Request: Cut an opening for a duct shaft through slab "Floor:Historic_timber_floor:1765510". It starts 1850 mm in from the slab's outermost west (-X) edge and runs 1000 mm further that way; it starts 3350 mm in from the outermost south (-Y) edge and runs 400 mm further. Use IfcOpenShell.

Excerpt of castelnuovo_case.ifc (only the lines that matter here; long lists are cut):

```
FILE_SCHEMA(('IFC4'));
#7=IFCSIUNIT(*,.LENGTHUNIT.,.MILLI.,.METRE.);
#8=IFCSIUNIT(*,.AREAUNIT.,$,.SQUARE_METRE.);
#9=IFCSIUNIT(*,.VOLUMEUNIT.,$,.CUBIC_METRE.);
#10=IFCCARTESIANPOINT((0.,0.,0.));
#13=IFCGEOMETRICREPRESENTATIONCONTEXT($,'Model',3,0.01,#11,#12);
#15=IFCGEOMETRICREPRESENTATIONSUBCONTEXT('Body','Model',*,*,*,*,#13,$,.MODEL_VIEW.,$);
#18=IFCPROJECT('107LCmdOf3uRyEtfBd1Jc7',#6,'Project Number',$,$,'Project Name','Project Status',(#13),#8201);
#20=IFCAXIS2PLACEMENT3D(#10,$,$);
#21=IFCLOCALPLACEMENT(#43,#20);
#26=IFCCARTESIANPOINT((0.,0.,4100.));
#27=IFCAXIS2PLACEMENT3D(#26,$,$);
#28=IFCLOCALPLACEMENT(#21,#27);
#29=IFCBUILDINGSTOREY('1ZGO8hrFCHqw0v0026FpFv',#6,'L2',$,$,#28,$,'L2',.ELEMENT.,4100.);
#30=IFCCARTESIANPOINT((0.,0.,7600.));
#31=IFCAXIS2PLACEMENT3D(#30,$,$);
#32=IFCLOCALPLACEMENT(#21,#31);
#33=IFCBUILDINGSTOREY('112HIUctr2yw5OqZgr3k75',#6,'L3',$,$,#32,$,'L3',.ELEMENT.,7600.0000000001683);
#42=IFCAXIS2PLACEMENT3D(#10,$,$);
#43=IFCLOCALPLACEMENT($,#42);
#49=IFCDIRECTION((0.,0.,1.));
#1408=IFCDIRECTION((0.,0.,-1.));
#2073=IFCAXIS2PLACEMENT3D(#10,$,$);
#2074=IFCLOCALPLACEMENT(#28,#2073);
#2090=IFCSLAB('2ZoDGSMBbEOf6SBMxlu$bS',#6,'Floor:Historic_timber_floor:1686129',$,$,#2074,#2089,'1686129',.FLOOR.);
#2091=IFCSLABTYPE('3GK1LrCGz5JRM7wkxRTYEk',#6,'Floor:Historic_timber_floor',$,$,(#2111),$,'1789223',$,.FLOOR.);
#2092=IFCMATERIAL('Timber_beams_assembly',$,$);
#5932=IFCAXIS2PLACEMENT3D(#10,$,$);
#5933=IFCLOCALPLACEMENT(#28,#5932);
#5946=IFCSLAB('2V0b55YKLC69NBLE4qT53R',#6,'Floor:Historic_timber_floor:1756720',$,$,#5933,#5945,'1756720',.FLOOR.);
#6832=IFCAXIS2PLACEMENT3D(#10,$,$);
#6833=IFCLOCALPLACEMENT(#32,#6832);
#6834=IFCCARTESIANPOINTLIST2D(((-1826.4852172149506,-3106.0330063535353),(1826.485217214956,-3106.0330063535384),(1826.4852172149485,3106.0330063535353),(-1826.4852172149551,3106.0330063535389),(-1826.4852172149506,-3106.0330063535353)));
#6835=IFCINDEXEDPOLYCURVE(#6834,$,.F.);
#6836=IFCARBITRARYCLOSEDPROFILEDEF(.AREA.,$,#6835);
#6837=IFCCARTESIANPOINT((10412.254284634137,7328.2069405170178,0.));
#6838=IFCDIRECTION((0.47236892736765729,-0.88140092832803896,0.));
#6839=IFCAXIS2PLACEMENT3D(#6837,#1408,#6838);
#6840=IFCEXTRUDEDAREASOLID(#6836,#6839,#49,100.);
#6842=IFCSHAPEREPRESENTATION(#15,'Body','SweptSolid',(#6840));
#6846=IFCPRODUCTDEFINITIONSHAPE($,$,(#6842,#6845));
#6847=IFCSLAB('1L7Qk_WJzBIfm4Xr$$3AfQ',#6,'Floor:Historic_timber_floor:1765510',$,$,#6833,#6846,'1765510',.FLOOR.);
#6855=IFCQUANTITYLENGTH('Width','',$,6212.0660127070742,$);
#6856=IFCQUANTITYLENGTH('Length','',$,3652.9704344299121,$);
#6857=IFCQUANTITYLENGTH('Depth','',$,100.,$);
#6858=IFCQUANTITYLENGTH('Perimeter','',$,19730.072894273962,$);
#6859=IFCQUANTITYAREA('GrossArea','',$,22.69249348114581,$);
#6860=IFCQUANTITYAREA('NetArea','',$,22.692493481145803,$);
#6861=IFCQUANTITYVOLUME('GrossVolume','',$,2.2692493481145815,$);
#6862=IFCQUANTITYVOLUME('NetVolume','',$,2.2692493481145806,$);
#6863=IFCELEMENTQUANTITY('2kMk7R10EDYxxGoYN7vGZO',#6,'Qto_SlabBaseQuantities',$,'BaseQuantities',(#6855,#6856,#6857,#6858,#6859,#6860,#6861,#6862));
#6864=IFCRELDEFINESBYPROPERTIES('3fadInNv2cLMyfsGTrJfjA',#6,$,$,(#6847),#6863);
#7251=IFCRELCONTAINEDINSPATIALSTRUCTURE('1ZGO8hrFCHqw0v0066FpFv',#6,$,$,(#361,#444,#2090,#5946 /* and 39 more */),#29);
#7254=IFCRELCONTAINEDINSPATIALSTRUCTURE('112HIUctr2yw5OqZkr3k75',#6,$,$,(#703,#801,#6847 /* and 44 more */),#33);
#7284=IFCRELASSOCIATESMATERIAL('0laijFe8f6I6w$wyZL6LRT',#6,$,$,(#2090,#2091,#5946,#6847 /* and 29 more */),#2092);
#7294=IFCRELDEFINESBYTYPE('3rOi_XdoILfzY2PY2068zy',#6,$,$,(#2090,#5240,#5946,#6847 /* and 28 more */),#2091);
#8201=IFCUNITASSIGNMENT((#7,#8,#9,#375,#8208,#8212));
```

```python
import numpy as np
import ifcopenshell
import ifcopenshell.api.feature
import ifcopenshell.api.geometry
import ifcopenshell.api.pset
import ifcopenshell.api.root
import ifcopenshell.geom
import ifcopenshell.util.element
import ifcopenshell.util.placement
import ifcopenshell.util.representation
import ifcopenshell.util.shape
import ifcopenshell.util.unit

model = ifcopenshell.open("castelnuovo_case.ifc")
unit_scale = ifcopenshell.util.unit.calculate_unit_scale(model)
area_scale = ifcopenshell.util.unit.calculate_unit_scale(model, "AREAUNIT")
volume_scale = ifcopenshell.util.unit.calculate_unit_scale(model, "VOLUMEUNIT")
settings = ifcopenshell.geom.settings()


def volume(element):
    """Net volume in cubic metres, openings subtracted."""
    shape = ifcopenshell.geom.create_shape(settings, element)
    return ifcopenshell.util.shape.get_volume(shape.geometry)


slab = model.by_id(6847)
before = volume(slab)

# Extent in the slab's own axes, in metres. The edges named are its -X and -Y sides.
slab_shape = ifcopenshell.geom.create_shape(settings, slab)
vertices = ifcopenshell.util.shape.get_vertices(slab_shape.geometry)
x_min, y_min, bottom = vertices.min(axis=0)
top = vertices[:, 2].max()

opening = ifcopenshell.api.root.create_entity(model, ifc_class="IfcOpeningElement", name="Duct shaft opening", predefined_type="OPENING")
context = ifcopenshell.util.representation.get_context(model, "Model", "Body", "MODEL_VIEW")
width, depth = 1, 0.4
outline = [(0.0, 0.0), (width, 0.0), (width, depth), (0.0, depth), (0.0, 0.0)]
# Overshoot both faces by 50 mm so the cut is clean.
shape = ifcopenshell.api.geometry.add_slab_representation(
    model, context=context, depth=top - bottom + 0.1, polyline=outline
)
ifcopenshell.api.geometry.assign_representation(model, product=opening, representation=shape)

matrix = ifcopenshell.util.placement.get_local_placement(slab.ObjectPlacement)
matrix[:, 3] = matrix @ np.append(np.array([x_min + 1.85, y_min + 3.35, bottom - 0.05]) / unit_scale, 1.0)
ifcopenshell.api.geometry.edit_object_placement(model, product=opening, matrix=matrix, is_si=False)
ifcopenshell.api.feature.add_feature(model, feature=opening, element=slab)

after = volume(slab)

# Update the slab's stored quantities.
qto = model.by_id(ifcopenshell.util.element.get_pset(slab, "Qto_SlabBaseQuantities", should_inherit=False)["id"])
ifcopenshell.api.pset.edit_qto(model, qto=qto, properties={
    "NetArea": after / (top - bottom) / area_scale,
    "NetVolume": after / volume_scale,
})

print(f"slab volume {before:.3f} -> {after:.3f} m3")

model.write("castelnuovo_case_rev.ifc")
```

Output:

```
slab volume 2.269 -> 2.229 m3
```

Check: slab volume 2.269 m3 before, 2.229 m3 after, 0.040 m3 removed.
